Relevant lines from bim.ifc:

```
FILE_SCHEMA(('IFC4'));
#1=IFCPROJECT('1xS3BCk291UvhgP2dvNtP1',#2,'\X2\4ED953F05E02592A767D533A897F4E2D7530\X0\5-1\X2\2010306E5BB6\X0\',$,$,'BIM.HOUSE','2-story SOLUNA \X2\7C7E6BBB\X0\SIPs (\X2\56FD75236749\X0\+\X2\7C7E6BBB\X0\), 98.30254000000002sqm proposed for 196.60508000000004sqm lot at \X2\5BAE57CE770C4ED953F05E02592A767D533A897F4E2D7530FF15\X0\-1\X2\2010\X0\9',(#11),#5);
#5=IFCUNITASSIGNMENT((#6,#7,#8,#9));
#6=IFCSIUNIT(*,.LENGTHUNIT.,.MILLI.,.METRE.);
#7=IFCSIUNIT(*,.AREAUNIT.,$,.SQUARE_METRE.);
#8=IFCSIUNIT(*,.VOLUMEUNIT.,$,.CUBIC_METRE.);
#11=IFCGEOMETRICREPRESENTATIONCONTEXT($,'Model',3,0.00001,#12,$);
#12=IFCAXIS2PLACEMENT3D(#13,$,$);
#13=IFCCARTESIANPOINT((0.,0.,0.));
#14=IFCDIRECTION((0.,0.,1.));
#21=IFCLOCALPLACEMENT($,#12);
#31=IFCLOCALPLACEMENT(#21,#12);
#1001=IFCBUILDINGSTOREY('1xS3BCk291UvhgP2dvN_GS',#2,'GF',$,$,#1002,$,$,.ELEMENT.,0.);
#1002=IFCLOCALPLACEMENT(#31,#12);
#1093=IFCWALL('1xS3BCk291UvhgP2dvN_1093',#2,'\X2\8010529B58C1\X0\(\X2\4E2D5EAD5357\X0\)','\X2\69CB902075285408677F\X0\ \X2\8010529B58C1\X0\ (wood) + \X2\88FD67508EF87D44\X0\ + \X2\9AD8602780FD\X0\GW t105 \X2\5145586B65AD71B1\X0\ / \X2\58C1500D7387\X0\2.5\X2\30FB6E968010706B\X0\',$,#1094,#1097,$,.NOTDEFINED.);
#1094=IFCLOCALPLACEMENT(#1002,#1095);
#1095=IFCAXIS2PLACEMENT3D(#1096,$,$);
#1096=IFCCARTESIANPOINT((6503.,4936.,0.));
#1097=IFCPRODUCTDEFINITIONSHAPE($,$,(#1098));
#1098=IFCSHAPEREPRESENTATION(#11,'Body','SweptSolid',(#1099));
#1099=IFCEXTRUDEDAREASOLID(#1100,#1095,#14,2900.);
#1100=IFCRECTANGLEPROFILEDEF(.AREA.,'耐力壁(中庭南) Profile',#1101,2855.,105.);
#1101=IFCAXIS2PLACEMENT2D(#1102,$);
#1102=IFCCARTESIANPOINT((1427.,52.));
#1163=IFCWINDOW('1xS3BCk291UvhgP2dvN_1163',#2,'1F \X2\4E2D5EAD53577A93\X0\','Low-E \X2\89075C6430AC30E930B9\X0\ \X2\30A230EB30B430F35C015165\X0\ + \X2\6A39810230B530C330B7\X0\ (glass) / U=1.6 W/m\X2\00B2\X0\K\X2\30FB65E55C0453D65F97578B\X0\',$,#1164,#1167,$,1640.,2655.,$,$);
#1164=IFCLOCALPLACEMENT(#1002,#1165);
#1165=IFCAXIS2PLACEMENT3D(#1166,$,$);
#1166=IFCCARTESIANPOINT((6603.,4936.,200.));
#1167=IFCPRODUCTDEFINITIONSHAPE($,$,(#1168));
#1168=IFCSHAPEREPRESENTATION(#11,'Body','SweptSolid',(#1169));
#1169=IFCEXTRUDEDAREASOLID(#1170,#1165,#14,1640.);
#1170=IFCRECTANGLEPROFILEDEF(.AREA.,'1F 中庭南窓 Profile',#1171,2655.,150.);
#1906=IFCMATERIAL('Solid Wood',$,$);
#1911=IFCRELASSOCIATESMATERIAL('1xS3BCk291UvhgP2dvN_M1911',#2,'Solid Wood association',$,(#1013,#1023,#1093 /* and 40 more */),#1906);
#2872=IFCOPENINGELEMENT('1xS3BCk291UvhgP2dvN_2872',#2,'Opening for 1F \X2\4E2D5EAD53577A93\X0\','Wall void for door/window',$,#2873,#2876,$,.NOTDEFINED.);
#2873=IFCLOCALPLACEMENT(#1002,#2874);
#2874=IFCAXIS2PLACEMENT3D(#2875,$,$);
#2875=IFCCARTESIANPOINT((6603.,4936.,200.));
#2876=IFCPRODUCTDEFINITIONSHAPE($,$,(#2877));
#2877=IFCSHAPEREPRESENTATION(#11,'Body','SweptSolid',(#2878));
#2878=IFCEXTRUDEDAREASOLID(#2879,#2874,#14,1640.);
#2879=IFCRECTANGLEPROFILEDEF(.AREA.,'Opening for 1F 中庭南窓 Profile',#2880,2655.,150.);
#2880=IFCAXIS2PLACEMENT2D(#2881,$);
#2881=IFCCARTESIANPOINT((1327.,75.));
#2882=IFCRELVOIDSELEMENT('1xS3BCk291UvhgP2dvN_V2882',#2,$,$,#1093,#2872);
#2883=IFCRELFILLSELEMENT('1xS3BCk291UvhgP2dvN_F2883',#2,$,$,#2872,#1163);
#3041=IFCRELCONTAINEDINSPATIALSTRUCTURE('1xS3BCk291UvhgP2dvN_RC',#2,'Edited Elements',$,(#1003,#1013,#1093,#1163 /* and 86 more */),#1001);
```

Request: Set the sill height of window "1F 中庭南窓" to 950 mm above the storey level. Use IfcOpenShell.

```python
import numpy as np
import ifcopenshell
import ifcopenshell.api.geometry
import ifcopenshell.geom
import ifcopenshell.util.element
import ifcopenshell.util.placement
import ifcopenshell.util.shape
import ifcopenshell.util.unit

model = ifcopenshell.open("bim.ifc")
unit_scale = ifcopenshell.util.unit.calculate_unit_scale(model)

window = model.by_guid("1xS3BCk291UvhgP2dvN_1163")
opening = window.FillsVoids[0].RelatingOpeningElement
storey = ifcopenshell.util.element.get_container(window, ifc_class="IfcBuildingStorey")
level = ifcopenshell.util.placement.get_local_placement(storey.ObjectPlacement)[2, 3]

# The opening's origin need not be at the sill, so measure its lowest point.
shape = ifcopenshell.geom.create_shape(ifcopenshell.geom.settings(), opening)
bottom = ifcopenshell.util.shape.get_shape_bottom_elevation(shape, shape.geometry) / unit_scale
dz = level + 0.95 / unit_scale - bottom

shift = np.array([0.0, 0.0, dz])
# The window is not placed relative to its opening, so move both.
for product in (opening, window):
    matrix = ifcopenshell.util.placement.get_local_placement(product.ObjectPlacement)
    matrix[:3, 3] += shift
    ifcopenshell.api.geometry.edit_object_placement(model, product=product, matrix=matrix, is_si=False)

print(f"moved by {dz * unit_scale:+.3f} m")

model.write("bim_rev.ifc")
```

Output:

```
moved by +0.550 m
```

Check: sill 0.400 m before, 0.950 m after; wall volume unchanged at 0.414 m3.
